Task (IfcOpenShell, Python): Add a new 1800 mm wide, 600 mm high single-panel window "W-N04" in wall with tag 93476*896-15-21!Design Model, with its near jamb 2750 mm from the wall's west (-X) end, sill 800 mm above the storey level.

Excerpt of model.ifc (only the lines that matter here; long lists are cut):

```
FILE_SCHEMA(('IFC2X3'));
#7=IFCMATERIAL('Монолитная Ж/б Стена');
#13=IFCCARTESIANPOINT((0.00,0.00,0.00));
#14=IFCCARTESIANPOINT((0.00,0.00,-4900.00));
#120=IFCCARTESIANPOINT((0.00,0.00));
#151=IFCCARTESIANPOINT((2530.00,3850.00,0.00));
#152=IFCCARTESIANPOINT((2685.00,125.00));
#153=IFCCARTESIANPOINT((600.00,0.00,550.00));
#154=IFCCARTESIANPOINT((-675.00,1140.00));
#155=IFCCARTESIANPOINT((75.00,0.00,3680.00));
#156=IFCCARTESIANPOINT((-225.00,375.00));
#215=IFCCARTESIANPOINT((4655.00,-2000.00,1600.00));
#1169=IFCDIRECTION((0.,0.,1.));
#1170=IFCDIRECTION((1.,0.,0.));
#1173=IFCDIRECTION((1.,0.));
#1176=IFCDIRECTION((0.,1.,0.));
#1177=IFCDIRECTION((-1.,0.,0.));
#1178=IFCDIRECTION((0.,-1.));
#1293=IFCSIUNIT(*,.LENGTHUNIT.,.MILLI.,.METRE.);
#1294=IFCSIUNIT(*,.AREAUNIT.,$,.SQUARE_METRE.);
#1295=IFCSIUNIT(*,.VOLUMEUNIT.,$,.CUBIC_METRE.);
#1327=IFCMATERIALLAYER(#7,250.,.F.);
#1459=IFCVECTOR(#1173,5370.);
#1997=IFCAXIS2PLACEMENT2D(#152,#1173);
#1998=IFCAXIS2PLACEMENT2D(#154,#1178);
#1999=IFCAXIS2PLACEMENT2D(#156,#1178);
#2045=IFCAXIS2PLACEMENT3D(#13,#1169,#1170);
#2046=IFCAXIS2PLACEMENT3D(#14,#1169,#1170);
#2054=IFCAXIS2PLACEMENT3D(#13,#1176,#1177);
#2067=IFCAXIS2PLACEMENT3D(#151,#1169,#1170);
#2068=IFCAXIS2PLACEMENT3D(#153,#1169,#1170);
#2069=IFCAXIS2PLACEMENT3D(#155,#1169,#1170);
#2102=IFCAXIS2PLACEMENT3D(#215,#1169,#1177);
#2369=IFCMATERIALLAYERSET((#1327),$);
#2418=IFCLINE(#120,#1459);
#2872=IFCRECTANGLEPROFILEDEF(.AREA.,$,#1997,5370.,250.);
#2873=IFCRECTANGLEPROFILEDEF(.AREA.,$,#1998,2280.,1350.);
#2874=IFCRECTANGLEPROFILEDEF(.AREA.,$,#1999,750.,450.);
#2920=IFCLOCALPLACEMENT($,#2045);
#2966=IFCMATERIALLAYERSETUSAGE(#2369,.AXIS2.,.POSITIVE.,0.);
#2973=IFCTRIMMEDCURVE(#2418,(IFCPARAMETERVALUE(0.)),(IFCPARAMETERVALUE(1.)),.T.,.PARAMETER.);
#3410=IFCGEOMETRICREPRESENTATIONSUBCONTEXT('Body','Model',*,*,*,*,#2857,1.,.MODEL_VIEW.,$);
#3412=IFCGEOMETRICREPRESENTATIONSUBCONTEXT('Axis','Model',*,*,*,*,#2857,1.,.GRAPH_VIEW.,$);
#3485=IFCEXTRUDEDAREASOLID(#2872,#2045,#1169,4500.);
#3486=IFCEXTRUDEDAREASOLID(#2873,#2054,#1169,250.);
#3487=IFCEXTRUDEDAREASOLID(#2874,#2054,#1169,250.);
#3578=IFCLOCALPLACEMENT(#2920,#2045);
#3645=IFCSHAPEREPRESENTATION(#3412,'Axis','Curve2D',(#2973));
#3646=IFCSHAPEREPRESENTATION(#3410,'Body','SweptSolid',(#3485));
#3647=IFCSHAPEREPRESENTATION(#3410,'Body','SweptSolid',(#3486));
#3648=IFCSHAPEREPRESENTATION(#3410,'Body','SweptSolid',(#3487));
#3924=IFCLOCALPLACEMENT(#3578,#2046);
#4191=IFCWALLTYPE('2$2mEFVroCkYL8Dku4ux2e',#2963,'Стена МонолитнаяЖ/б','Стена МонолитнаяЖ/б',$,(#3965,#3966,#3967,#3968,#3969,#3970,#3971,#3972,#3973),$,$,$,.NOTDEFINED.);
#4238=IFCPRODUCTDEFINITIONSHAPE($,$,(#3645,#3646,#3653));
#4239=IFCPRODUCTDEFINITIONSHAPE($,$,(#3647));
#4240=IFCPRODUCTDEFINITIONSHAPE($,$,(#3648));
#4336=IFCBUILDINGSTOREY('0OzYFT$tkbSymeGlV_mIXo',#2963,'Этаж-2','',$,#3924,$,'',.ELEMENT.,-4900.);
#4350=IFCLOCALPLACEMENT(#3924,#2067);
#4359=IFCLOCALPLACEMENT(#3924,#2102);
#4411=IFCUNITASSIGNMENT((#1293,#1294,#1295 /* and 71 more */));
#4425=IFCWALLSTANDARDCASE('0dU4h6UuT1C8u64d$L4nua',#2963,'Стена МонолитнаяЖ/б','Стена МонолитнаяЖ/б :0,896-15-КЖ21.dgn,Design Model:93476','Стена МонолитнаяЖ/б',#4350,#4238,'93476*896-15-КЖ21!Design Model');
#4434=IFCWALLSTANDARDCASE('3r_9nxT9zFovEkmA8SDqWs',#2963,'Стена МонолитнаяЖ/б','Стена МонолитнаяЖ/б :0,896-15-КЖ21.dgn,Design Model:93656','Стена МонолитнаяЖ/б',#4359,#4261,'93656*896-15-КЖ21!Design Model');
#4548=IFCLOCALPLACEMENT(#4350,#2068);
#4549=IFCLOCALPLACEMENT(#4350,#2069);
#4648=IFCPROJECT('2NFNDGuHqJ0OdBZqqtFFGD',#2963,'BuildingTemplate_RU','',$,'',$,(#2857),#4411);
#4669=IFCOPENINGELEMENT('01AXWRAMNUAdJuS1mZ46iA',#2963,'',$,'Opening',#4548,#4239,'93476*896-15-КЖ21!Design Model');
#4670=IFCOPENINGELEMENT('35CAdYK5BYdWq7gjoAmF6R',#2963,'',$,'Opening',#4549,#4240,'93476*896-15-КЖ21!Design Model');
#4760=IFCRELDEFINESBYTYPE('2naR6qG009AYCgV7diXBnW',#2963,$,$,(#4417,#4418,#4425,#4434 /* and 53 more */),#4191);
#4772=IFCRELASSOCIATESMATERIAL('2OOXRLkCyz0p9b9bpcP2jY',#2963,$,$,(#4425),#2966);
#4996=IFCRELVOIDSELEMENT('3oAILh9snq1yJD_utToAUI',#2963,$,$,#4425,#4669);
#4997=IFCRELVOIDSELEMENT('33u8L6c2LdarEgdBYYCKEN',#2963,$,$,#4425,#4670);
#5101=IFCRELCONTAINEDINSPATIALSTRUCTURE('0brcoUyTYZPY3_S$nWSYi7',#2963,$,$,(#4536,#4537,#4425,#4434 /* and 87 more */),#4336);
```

```python
import numpy as np
import ifcopenshell
import ifcopenshell.api.feature
import ifcopenshell.api.geometry
import ifcopenshell.api.root
import ifcopenshell.api.spatial
import ifcopenshell.api.type
import ifcopenshell.geom
import ifcopenshell.util.element
import ifcopenshell.util.placement
import ifcopenshell.util.representation
import ifcopenshell.util.shape
import ifcopenshell.util.unit

model = ifcopenshell.open("model.ifc")
unit_scale = ifcopenshell.util.unit.calculate_unit_scale(model)
settings = ifcopenshell.geom.settings()


def volume(element):
    """Net volume in cubic metres, openings subtracted."""
    shape = ifcopenshell.geom.create_shape(settings, element)
    return ifcopenshell.util.shape.get_volume(shape.geometry)


wall = model.by_guid("0dU4h6UuT1C8u64d$L4nua")
storey = ifcopenshell.util.element.get_container(wall, ifc_class="IfcBuildingStorey")
context = ifcopenshell.util.representation.get_context(model, "Model", "Body", "MODEL_VIEW")
before = volume(wall)

width, height, from_end, sill = 1.8, 0.6, 2.75, 0.8  # metres

# The wall runs along its own X axis, and the end named is its -X end.
wall_shape = ifcopenshell.geom.create_shape(settings, wall)
x, y, z = ifcopenshell.util.shape.get_vertices(wall_shape.geometry).T
start = x.min() + from_end
face, thickness = float(y.min()), float(y.max() - y.min())
wall_matrix = ifcopenshell.util.placement.get_local_placement(wall.ObjectPlacement)
level = ifcopenshell.util.placement.get_local_placement(storey.ObjectPlacement)[2, 3]


def in_wall(x, y):
    """Placement at x, y metres in the wall's axes, at sill height."""
    matrix = wall_matrix.copy()
    matrix[:, 3] = wall_matrix @ np.array([x / unit_scale, y / unit_scale, 0.0, 1.0])
    matrix[2, 3] = level + sill / unit_scale
    return matrix


# Opening: a box that overshoots both wall faces by 50 mm.
opening = ifcopenshell.api.root.create_entity(model, ifc_class="IfcOpeningElement")
box = ifcopenshell.api.geometry.add_wall_representation(
    model, context=context, length=width, height=height, thickness=thickness + 0.1
)
ifcopenshell.api.geometry.assign_representation(model, product=opening, representation=box)
ifcopenshell.api.geometry.edit_object_placement(model, product=opening, matrix=in_wall(start, face - 0.05), is_si=False)
ifcopenshell.api.feature.add_feature(model, feature=opening, element=wall)

window = ifcopenshell.api.root.create_entity(model, ifc_class="IfcWindow", name="W-N04")
window.OverallWidth, window.OverallHeight = width / unit_scale, height / unit_scale
body = ifcopenshell.api.geometry.add_window_representation(
    model,
    context=context,
    overall_width=window.OverallWidth,
    overall_height=window.OverallHeight,
    partition_type="SINGLE_PANEL",
)
ifcopenshell.api.geometry.assign_representation(model, product=window, representation=body)
ifcopenshell.api.spatial.assign_container(model, products=[window], relating_structure=storey)
fills = ifcopenshell.api.feature.add_filling(model, opening=opening, element=window)
fills.OwnerHistory = window.OwnerHistory  # required in IFC2X3

# IFC2X3 keeps the operation on the window style.
style = ifcopenshell.api.root.create_entity(model, ifc_class="IfcWindowStyle", name="W-N04")
style.OperationType, style.ConstructionType = "SINGLE_PANEL", "NOTDEFINED"
style.ParameterTakesPrecedence = style.Sizeable = False
ifcopenshell.api.type.assign_type(model, related_objects=[window], relating_type=style)

# Centre the window in the wall's thickness.
ifcopenshell.api.geometry.edit_object_placement(model, product=window, matrix=in_wall(start, face), is_si=False)
window_shape = ifcopenshell.geom.create_shape(settings, window)
depth = ifcopenshell.util.shape.get_vertices(window_shape.geometry)[:, 1]
offset = face + thickness / 2 - (depth.min() + depth.max()) / 2
ifcopenshell.api.geometry.edit_object_placement(model, product=window, matrix=in_wall(start, offset), is_si=False)

after = volume(wall)

print(f"wall volume {before:.3f} -> {after:.3f} m3")

model.write("model_edited.ifc")
```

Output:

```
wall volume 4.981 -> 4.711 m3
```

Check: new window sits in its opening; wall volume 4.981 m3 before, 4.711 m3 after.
